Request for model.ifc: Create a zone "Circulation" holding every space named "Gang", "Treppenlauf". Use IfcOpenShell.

First a look at what the model holds.

```python
import ifcopenshell

model = ifcopenshell.open("model.ifc")
print(model.schema)
seen = {}
for space in model.by_type("IfcSpace"):
    seen[space.LongName] = seen.get(space.LongName, 0) + 1
for name, count in sorted(seen.items(), key=str):
    print(count, "x", name)
print("zones:", [z.Name for z in model.by_type("IfcZone")][:20])
```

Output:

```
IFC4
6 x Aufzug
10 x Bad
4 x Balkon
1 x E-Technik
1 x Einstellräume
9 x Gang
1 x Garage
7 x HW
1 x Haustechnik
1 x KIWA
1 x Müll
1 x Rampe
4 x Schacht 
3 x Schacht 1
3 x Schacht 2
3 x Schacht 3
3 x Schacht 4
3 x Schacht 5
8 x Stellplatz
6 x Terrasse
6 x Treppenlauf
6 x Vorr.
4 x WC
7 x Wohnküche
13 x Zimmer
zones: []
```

```python
import ifcopenshell
import ifcopenshell.api.group
import ifcopenshell.api.root

model = ifcopenshell.open("model.ifc")

names = {"Gang", "Treppenlauf"}
spaces = [s for s in model.by_type("IfcSpace") if s.LongName in names]

zone = ifcopenshell.api.root.create_entity(model, ifc_class="IfcZone", name="Circulation")
ifcopenshell.api.group.assign_group(model, products=spaces, group=zone)
print(len(spaces), "spaces in", zone.Name)

model.write("model-out.ifc")
```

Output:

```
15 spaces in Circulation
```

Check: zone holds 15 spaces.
